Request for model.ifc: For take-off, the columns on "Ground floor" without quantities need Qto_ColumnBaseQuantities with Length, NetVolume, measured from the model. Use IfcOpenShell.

First a look at what the model holds.

```python
import ifcopenshell
import ifcopenshell.util.element
import ifcopenshell.util.unit

model = ifcopenshell.open("model.ifc")
print(model.schema)
for unit_type in ("LENGTHUNIT", "AREAUNIT", "VOLUMEUNIT"):
    print(unit_type, ifcopenshell.util.unit.calculate_unit_scale(model, unit_type))
storey = next(s for s in model.by_type("IfcBuildingStorey") if s.Name == "Ground floor")
columns = [e for e in ifcopenshell.util.element.get_decomposition(storey) if e.is_a("IfcColumn")]
for e in sorted(columns, key=lambda e: e.id()):
    print(e.id(), e.is_a(), e.Name, list(ifcopenshell.util.element.get_psets(e, qtos_only=True)), sep=" | ")
```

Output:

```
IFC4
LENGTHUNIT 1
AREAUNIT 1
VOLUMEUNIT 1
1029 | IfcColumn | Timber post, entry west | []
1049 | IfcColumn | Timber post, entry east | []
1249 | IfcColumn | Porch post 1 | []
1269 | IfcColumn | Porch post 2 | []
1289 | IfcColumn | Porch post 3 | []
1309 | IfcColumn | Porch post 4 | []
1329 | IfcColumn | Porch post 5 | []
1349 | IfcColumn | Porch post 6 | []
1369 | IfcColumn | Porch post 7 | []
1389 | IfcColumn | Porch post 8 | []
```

```python
import ifcopenshell
import ifcopenshell.api.pset
import ifcopenshell.geom
import ifcopenshell.util.element
import ifcopenshell.util.shape
import ifcopenshell.util.unit

model = ifcopenshell.open("model.ifc")
unit_scale = ifcopenshell.util.unit.calculate_unit_scale(model)
volume_scale = ifcopenshell.util.unit.calculate_unit_scale(model, "VOLUMEUNIT")
settings = ifcopenshell.geom.settings()

storey = next(s for s in model.by_type("IfcBuildingStorey") if s.Name == "Ground floor")
columns = [e for e in ifcopenshell.util.element.get_decomposition(storey) if e.is_a("IfcColumn")]

for e in sorted(columns, key=lambda e: e.id()):
    if ifcopenshell.util.element.get_psets(e, qtos_only=True, should_inherit=False):
        continue
    # Geometry comes back in metres, in the element's own axes.
    shape = ifcopenshell.geom.create_shape(settings, e)
    values = {
        "Length": ifcopenshell.util.shape.get_z(shape.geometry) / unit_scale,
        "NetVolume": ifcopenshell.util.shape.get_volume(shape.geometry) / volume_scale,
    }
    qto = ifcopenshell.api.pset.add_qto(model, product=e, name="Qto_ColumnBaseQuantities")
    ifcopenshell.api.pset.edit_qto(model, qto=qto, properties=values)
    print(e.id(), {k: round(v, 3) for k, v in values.items()})

model.write("model_v2.ifc")
```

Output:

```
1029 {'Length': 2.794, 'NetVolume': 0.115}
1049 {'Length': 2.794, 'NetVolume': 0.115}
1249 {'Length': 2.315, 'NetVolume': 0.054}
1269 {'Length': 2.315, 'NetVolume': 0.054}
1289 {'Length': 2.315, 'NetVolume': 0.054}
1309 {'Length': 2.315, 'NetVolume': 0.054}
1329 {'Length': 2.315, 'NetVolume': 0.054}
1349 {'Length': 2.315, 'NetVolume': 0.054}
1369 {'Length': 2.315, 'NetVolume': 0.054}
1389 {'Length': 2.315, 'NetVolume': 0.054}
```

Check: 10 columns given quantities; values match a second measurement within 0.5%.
